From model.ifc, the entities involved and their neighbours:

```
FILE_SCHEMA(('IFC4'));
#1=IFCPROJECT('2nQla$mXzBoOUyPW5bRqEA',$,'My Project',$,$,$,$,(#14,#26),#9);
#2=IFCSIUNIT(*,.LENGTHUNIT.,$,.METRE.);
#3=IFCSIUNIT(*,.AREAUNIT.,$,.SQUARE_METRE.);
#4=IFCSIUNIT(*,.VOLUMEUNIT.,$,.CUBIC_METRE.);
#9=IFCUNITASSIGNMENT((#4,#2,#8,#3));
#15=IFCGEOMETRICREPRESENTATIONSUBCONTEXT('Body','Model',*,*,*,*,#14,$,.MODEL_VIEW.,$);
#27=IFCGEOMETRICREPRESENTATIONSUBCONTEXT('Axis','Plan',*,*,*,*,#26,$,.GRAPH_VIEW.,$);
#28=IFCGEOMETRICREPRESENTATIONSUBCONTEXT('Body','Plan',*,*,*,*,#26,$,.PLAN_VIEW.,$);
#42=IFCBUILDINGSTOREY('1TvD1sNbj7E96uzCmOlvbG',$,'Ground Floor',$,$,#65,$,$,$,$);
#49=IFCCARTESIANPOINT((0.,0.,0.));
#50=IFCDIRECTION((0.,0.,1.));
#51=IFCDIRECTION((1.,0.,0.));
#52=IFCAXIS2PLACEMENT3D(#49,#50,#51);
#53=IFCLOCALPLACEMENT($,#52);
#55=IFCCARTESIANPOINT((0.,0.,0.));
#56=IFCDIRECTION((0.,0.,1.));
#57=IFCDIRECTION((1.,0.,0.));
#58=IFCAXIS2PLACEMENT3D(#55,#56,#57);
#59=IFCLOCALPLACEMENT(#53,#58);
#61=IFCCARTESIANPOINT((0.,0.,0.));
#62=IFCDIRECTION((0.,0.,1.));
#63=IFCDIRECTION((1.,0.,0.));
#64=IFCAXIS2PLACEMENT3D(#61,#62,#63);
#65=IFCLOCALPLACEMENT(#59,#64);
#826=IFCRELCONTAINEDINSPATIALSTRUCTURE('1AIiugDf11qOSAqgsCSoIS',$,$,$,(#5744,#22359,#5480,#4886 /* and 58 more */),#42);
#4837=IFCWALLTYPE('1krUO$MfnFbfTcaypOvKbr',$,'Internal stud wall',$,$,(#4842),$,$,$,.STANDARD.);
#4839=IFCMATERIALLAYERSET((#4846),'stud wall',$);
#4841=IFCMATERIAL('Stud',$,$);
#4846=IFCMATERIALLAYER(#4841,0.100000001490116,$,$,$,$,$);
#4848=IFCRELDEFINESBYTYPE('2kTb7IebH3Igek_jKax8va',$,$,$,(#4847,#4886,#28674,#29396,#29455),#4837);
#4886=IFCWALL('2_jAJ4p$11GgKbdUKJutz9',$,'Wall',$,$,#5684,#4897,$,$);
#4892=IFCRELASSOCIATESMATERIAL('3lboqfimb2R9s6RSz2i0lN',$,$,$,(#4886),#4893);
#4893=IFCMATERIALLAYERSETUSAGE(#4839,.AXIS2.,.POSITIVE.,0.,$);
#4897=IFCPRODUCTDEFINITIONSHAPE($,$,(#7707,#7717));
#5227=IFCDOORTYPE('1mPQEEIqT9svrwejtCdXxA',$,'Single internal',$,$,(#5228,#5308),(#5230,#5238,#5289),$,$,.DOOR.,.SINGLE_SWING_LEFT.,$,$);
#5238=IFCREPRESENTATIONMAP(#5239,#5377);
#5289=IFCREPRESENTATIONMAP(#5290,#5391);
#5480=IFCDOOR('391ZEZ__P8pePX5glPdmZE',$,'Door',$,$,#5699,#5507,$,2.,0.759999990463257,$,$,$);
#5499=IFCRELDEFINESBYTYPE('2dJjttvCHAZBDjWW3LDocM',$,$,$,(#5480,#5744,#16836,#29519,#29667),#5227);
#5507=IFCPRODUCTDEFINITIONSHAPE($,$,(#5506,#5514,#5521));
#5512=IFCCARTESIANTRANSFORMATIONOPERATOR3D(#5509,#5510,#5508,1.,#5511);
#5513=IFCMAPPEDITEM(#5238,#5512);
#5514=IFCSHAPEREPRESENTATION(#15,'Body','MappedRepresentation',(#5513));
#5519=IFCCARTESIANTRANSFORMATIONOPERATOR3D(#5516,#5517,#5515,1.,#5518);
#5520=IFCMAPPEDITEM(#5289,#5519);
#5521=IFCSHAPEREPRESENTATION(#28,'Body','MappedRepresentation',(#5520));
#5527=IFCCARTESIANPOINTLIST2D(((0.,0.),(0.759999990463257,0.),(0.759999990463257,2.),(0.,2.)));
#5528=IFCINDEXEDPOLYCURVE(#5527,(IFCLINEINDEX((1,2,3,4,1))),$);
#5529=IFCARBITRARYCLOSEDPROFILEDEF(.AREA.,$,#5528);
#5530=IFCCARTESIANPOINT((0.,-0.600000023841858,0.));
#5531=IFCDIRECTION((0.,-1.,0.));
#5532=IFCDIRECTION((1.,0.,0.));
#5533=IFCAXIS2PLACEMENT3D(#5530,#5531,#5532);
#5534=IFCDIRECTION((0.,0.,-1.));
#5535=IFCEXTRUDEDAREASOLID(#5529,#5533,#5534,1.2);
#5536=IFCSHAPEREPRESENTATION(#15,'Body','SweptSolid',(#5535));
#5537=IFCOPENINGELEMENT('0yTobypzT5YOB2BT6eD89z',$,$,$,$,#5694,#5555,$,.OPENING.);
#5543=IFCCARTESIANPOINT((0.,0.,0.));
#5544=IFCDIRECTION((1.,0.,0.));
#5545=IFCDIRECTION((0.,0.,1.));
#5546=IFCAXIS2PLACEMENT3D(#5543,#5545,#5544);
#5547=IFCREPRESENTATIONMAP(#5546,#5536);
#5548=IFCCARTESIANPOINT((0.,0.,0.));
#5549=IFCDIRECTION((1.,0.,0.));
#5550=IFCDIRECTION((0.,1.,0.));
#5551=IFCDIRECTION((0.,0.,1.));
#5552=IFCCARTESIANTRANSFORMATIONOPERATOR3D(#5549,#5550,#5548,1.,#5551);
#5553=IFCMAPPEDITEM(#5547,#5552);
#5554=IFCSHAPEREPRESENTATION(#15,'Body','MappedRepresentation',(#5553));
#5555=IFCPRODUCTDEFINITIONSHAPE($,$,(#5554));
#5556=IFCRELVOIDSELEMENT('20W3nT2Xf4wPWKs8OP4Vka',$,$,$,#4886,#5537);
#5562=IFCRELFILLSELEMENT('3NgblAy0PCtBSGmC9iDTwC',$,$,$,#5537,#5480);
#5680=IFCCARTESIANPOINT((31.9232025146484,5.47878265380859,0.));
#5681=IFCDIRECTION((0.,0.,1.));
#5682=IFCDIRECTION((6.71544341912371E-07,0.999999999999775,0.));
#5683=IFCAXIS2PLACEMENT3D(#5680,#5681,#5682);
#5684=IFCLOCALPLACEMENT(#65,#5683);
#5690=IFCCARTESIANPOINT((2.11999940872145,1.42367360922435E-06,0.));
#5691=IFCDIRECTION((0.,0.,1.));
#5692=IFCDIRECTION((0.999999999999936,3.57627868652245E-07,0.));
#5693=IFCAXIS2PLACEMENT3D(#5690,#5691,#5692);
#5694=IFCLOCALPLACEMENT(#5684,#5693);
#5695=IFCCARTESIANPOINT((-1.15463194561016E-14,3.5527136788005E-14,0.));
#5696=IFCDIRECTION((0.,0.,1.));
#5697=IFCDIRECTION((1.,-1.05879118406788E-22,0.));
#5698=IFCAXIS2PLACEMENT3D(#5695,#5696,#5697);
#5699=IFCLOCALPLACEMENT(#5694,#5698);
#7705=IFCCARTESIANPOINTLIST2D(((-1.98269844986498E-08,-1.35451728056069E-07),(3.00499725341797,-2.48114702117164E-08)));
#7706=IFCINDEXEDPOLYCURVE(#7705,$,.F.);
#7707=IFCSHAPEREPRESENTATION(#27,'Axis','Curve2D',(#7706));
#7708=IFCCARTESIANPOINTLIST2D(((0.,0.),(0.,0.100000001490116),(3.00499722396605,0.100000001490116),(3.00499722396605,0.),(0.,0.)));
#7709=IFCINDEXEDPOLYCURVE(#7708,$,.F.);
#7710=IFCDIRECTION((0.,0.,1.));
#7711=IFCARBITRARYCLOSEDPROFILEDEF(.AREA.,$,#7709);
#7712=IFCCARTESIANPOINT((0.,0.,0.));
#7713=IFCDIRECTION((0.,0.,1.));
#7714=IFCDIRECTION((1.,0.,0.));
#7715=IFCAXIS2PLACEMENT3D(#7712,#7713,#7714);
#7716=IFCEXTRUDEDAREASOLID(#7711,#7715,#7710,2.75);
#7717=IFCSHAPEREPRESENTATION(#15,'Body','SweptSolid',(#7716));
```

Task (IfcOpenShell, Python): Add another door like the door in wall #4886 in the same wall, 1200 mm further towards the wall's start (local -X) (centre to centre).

```python
import ifcopenshell
import ifcopenshell.api.feature
import ifcopenshell.api.geometry
import ifcopenshell.api.root
import ifcopenshell.geom
import ifcopenshell.util.element
import ifcopenshell.util.placement
import ifcopenshell.util.shape

model = ifcopenshell.open("model.ifc")
settings = ifcopenshell.geom.settings()


def volume(element):
    """Net volume in cubic metres, openings subtracted."""
    shape = ifcopenshell.geom.create_shape(settings, element)
    return ifcopenshell.util.shape.get_volume(shape.geometry)


door = model.by_id(5480)
opening = door.FillsVoids[0].RelatingOpeningElement
wall = opening.VoidsElements[0].RelatingBuildingElement
before = volume(wall)
shift = ifcopenshell.util.placement.get_local_placement(wall.ObjectPlacement)[:3, 0] * -1.2

# copy_class copies the void relationship, type, container and properties, but no geometry.
new_opening = ifcopenshell.api.root.copy_class(model, product=opening)
new_opening.Representation = ifcopenshell.util.element.copy_deep(
    model, opening.Representation, exclude=["IfcGeometricRepresentationContext", "IfcRepresentationMap"]
)
new_door = ifcopenshell.api.root.copy_class(model, product=door)
new_door.Representation = ifcopenshell.util.element.copy_deep(
    model, door.Representation, exclude=["IfcGeometricRepresentationContext", "IfcRepresentationMap"]
)
ifcopenshell.api.feature.add_filling(model, opening=new_opening, element=new_door)

for old, new in ((opening, new_opening), (door, new_door)):
    matrix = ifcopenshell.util.placement.get_local_placement(old.ObjectPlacement)
    matrix[:3, 3] += shift
    ifcopenshell.api.geometry.edit_object_placement(model, product=new, matrix=matrix, is_si=False)

after = volume(wall)

print(f"wall volume {before:.3f} -> {after:.3f} m3")

model.write("model_updated.ifc")
```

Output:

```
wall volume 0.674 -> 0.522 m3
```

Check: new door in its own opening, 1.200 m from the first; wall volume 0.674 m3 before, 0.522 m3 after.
